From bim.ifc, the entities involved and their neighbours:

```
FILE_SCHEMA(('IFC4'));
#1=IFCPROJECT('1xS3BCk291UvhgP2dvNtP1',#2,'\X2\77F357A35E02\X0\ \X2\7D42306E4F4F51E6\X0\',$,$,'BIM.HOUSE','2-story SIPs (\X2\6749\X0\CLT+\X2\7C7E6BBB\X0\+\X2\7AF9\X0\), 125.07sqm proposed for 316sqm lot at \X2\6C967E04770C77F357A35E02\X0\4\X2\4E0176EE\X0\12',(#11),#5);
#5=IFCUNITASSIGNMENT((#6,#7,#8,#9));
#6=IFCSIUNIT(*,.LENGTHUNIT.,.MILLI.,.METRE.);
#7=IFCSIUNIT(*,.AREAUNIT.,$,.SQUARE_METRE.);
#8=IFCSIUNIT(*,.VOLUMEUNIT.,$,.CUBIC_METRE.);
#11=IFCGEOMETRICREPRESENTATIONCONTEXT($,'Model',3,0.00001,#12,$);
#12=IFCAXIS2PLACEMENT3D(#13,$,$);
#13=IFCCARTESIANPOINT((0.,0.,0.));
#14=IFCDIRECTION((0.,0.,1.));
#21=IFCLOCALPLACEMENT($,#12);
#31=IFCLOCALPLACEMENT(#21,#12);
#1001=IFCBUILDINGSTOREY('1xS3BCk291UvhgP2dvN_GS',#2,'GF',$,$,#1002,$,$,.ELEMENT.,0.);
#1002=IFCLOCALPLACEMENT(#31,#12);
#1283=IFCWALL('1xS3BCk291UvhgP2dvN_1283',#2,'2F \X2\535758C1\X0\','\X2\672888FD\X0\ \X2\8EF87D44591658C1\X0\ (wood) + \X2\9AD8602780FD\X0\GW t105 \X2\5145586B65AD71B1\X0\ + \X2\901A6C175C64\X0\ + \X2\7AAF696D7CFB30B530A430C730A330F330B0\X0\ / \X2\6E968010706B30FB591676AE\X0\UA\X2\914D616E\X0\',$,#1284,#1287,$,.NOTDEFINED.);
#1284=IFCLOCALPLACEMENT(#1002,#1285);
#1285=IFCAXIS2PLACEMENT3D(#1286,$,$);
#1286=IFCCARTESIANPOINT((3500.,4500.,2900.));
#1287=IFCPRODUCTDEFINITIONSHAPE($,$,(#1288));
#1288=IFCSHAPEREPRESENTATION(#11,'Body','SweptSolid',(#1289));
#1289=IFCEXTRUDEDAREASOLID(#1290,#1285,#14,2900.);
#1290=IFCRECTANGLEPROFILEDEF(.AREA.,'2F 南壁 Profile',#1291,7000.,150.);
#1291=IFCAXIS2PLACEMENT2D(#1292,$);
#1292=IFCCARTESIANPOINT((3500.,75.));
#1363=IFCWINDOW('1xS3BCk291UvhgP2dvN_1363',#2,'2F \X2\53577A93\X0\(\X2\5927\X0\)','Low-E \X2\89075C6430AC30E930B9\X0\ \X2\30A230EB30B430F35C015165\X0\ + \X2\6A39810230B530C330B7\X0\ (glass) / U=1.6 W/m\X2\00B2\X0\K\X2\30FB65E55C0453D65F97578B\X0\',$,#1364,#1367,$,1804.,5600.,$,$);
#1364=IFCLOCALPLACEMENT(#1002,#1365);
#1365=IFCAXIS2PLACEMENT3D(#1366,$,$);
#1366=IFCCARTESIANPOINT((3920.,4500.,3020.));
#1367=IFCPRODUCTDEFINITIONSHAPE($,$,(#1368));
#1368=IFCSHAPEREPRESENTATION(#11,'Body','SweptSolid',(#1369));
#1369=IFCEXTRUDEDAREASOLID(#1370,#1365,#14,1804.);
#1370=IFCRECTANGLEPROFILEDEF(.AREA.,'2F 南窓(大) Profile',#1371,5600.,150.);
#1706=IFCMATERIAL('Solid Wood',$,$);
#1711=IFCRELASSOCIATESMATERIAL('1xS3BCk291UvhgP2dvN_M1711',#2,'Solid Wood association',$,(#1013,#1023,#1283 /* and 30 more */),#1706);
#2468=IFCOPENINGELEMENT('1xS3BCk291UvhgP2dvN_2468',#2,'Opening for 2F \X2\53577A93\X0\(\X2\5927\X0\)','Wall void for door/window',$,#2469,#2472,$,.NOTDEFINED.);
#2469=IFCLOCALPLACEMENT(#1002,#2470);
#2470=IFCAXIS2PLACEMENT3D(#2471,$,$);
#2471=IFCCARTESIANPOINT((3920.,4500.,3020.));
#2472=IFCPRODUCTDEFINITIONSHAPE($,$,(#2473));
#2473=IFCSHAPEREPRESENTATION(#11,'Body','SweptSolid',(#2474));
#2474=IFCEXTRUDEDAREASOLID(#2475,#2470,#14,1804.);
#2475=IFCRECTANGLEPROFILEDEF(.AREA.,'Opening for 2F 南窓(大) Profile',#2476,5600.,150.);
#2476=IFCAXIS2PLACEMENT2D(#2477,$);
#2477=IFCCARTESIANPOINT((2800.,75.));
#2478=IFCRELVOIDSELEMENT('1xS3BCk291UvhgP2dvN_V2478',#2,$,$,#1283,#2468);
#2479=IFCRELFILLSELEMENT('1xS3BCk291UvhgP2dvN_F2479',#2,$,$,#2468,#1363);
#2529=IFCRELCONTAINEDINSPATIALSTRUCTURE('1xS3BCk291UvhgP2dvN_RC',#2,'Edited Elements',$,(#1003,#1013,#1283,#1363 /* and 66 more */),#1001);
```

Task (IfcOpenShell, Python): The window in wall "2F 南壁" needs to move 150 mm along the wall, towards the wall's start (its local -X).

```python
import ifcopenshell
import ifcopenshell.api.geometry
import ifcopenshell.util.placement
import ifcopenshell.util.unit

model = ifcopenshell.open("bim.ifc")
unit_scale = ifcopenshell.util.unit.calculate_unit_scale(model)

window = model.by_id(1363)
opening = window.FillsVoids[0].RelatingOpeningElement
wall = opening.VoidsElements[0].RelatingBuildingElement

wall_matrix = ifcopenshell.util.placement.get_local_placement(wall.ObjectPlacement)
shift = wall_matrix[:3, 0] * -0.15 / unit_scale
before = ifcopenshell.util.placement.get_local_placement(window.ObjectPlacement)[:3, 3].copy()

# The window is not placed relative to its opening, so move both.
for product in (opening, window):
    matrix = ifcopenshell.util.placement.get_local_placement(product.ObjectPlacement)
    matrix[:3, 3] += shift
    ifcopenshell.api.geometry.edit_object_placement(model, product=product, matrix=matrix, is_si=False)

after = ifcopenshell.util.placement.get_local_placement(window.ObjectPlacement)[:3, 3]
print("window moved by", (after - before).round(3) + 0.0)

model.write("bim_rev.ifc")
```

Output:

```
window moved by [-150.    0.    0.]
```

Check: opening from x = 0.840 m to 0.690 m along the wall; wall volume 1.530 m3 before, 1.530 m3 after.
